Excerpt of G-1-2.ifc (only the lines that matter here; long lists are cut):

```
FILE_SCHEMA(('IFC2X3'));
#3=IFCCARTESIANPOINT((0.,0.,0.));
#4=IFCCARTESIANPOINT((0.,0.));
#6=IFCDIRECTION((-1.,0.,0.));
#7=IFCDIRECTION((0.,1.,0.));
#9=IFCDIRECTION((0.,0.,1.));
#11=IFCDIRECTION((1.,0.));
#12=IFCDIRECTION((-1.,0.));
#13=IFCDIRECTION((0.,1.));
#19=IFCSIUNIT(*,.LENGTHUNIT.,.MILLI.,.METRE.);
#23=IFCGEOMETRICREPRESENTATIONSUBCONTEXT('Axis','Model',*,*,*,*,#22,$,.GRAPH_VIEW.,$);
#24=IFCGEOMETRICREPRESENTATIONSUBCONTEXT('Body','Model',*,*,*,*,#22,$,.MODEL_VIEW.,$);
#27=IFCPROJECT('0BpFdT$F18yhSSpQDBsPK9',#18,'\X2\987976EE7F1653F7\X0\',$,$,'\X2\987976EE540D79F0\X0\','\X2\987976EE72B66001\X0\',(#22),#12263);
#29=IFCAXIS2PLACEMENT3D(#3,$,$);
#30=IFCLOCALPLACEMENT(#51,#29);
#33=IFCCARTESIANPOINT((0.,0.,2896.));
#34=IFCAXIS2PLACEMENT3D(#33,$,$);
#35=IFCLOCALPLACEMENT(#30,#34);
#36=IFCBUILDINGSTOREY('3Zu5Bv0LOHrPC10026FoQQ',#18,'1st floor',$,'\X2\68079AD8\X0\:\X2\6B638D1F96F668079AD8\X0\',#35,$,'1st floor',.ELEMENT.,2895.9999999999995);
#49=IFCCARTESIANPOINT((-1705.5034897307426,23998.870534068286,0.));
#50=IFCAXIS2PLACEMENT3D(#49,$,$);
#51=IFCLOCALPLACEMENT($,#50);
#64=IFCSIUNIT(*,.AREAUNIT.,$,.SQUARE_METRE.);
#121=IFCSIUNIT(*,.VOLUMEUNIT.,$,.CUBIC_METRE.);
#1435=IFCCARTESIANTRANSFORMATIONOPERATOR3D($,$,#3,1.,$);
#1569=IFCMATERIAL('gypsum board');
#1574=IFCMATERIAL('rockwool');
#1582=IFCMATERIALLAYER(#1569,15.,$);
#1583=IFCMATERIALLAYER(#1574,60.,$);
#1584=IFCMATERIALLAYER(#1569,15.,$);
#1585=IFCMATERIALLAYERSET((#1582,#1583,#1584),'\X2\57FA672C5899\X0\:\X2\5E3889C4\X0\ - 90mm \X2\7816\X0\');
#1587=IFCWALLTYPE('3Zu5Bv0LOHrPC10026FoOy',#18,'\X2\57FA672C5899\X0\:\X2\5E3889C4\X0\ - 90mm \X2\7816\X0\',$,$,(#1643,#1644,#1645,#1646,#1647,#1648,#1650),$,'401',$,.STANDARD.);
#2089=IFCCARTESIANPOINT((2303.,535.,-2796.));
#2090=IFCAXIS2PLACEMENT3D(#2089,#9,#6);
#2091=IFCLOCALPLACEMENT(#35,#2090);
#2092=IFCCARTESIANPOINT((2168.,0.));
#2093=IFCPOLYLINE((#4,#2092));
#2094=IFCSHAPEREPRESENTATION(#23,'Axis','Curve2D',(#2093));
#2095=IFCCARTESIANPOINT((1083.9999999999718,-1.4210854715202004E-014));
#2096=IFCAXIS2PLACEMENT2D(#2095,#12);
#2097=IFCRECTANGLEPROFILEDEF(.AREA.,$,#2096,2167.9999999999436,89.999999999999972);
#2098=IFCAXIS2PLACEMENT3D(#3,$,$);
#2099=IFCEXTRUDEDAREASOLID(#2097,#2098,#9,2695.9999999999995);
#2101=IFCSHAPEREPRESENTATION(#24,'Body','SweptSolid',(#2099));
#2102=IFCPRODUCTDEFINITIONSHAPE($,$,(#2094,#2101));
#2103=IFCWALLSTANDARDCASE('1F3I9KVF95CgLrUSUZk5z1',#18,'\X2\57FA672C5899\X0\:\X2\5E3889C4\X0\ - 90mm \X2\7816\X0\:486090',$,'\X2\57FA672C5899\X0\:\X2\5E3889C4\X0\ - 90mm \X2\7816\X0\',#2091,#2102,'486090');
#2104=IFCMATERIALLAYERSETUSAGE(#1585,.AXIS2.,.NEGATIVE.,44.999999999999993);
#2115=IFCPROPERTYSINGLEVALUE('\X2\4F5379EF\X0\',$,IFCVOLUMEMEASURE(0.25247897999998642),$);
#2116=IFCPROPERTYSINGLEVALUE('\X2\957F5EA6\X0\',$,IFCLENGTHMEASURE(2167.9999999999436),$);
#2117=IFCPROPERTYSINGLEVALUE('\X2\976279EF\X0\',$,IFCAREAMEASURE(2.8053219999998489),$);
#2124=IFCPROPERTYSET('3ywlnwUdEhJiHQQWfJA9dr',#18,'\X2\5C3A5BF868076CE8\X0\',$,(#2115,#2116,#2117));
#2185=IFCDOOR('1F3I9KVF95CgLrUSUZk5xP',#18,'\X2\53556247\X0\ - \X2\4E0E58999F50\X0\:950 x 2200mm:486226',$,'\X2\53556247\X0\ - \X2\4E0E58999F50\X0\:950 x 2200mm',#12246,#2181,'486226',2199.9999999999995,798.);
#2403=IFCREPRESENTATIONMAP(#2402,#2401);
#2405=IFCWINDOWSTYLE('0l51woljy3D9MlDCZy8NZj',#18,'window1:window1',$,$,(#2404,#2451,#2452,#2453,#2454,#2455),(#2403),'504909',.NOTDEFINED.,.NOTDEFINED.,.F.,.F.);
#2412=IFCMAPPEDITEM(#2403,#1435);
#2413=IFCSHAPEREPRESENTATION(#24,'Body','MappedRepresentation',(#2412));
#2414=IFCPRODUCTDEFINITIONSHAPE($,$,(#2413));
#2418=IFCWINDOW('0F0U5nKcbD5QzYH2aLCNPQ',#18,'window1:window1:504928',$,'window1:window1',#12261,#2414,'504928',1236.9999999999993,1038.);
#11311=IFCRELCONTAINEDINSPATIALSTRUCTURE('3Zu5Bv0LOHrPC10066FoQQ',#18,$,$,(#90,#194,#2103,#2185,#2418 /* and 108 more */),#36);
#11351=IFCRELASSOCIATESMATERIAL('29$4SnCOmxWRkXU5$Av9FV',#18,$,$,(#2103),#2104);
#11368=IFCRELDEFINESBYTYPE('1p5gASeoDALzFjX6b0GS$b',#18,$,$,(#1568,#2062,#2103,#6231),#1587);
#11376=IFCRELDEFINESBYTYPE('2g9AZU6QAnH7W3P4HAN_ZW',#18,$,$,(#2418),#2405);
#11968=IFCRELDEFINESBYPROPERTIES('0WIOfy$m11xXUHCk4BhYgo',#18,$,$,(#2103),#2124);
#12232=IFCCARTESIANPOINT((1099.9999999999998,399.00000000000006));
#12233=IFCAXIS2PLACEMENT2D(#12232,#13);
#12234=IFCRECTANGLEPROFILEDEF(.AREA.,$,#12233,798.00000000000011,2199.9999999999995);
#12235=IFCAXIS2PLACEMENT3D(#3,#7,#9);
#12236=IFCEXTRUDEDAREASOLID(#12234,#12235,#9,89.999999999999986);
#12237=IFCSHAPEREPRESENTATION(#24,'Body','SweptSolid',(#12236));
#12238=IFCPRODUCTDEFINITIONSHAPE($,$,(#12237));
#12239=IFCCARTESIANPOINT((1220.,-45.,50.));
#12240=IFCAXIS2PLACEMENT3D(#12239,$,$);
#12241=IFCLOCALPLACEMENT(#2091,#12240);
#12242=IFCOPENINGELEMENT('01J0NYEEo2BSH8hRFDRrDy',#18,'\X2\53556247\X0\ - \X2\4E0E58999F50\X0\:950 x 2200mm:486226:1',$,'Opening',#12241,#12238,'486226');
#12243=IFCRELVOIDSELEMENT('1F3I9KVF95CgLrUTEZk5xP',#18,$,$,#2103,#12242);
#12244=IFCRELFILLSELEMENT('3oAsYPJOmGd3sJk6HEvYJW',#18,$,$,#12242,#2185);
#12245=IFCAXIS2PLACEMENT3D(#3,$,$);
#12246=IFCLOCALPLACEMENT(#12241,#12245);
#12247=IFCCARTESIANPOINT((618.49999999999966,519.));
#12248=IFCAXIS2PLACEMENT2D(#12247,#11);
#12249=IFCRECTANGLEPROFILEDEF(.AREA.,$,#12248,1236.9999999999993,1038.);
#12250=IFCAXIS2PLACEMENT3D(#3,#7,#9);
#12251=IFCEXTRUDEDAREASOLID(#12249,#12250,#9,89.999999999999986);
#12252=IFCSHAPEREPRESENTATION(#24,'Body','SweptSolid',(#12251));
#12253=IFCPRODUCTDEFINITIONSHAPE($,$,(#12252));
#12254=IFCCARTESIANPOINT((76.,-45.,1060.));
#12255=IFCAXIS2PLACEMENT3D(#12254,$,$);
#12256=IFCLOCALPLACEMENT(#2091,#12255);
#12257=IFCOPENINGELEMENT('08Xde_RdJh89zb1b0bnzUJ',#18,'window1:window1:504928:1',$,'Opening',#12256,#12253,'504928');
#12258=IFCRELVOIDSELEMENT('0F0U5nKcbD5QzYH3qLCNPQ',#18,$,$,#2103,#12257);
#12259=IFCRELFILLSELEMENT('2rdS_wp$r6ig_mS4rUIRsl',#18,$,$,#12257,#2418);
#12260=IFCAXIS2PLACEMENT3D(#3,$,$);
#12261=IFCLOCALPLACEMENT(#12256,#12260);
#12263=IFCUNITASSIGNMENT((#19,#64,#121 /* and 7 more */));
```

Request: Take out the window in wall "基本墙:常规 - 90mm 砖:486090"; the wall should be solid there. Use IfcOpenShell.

```python
import ifcopenshell
import ifcopenshell.api.feature
import ifcopenshell.api.pset
import ifcopenshell.api.root
import ifcopenshell.geom
import ifcopenshell.util.element
import ifcopenshell.util.shape
import ifcopenshell.util.unit

model = ifcopenshell.open("G-1-2.ifc")
area_scale = ifcopenshell.util.unit.calculate_unit_scale(model, "AREAUNIT")
volume_scale = ifcopenshell.util.unit.calculate_unit_scale(model, "VOLUMEUNIT")
settings = ifcopenshell.geom.settings()


def volume(element):
    """Net volume in cubic metres, openings subtracted."""
    shape = ifcopenshell.geom.create_shape(settings, element)
    return ifcopenshell.util.shape.get_volume(shape.geometry)


window = model.by_guid("0F0U5nKcbD5QzYH2aLCNPQ")
opening = window.FillsVoids[0].RelatingOpeningElement
wall = opening.VoidsElements[0].RelatingBuildingElement
before = volume(wall)

ifcopenshell.api.root.remove_product(model, product=window)
ifcopenshell.api.feature.remove_feature(model, feature=opening)

after = volume(wall)
thickness = 0.09  # wall thickness in metres

# Update the wall's stored quantities.
pset = model.by_id(ifcopenshell.util.element.get_pset(wall, "尺寸标注", should_inherit=False)["id"])
ifcopenshell.api.pset.edit_pset(model, pset=pset, properties={
    "体积": model.create_entity("IfcVolumeMeasure", after / volume_scale),
    "面积": model.create_entity("IfcAreaMeasure", after / thickness / area_scale),
})

print(f"wall volume {before:.3f} -> {after:.3f} m3")

model.write("G-1-2_rev.ifc")
```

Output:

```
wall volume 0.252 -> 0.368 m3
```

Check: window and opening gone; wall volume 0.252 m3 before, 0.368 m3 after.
